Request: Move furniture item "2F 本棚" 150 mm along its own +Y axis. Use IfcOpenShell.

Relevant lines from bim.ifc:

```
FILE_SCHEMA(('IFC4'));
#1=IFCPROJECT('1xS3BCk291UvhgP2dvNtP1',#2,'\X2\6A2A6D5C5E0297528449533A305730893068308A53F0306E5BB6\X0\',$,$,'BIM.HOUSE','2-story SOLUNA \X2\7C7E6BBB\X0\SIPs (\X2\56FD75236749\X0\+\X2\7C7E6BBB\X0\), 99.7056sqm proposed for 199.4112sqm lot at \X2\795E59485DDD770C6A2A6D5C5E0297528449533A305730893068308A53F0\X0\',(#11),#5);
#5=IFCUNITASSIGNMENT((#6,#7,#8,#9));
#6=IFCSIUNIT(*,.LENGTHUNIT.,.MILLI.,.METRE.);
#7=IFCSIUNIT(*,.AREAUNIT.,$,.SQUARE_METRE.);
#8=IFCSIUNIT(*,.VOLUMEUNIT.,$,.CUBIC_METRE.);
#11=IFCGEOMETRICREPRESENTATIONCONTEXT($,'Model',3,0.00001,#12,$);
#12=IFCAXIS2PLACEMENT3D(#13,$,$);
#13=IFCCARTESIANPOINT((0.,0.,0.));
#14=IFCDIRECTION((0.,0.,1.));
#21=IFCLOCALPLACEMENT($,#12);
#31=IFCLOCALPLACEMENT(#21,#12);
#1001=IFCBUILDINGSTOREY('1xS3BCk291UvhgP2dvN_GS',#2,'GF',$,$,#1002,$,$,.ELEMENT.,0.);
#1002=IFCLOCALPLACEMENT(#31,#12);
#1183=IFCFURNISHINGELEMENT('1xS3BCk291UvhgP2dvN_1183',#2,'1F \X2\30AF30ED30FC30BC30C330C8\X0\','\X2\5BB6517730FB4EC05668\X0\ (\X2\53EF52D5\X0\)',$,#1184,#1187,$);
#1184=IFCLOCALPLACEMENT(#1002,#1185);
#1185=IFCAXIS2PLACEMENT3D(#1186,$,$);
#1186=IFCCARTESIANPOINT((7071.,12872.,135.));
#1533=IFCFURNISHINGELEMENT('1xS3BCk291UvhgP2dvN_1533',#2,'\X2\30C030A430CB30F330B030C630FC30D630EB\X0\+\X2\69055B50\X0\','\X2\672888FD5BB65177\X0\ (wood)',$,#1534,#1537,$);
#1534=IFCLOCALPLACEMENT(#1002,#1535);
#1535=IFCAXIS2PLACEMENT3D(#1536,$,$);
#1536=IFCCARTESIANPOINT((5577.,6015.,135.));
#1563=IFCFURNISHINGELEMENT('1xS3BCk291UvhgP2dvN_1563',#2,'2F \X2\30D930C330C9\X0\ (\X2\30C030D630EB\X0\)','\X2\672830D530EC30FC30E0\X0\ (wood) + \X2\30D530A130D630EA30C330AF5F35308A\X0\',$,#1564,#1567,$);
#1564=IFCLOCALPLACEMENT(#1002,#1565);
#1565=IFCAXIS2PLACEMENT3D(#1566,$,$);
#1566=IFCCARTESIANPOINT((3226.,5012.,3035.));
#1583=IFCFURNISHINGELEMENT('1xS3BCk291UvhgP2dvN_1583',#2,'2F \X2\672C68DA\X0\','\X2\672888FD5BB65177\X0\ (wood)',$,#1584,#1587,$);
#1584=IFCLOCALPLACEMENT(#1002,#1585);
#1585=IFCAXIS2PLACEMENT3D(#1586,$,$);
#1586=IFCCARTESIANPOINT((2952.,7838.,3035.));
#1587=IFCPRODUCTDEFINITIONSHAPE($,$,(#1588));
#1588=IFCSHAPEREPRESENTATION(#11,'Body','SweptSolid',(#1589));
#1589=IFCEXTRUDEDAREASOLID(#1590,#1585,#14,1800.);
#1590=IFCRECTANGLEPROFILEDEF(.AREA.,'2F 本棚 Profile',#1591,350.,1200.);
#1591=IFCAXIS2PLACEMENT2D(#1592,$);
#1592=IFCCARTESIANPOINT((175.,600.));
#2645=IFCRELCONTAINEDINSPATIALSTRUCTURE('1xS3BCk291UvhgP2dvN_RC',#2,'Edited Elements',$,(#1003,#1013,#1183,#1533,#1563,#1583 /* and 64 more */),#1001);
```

```python
import ifcopenshell
import ifcopenshell.api.geometry
import ifcopenshell.util.placement
import ifcopenshell.util.unit

model = ifcopenshell.open("bim.ifc")
unit_scale = ifcopenshell.util.unit.calculate_unit_scale(model)

item = model.by_id(1583)
matrix = ifcopenshell.util.placement.get_local_placement(item.ObjectPlacement)
matrix[:3, 3] += matrix[:3, 1] * 0.15 / unit_scale
ifcopenshell.api.geometry.edit_object_placement(model, product=item, matrix=matrix, is_si=False)

print(ifcopenshell.util.placement.get_local_placement(item.ObjectPlacement).round(3) + 0.0)

model.write("bim_edited.ifc")
```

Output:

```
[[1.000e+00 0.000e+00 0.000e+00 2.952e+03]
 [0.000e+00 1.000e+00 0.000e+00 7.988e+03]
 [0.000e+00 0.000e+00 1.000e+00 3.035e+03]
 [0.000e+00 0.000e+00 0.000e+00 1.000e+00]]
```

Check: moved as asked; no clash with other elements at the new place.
